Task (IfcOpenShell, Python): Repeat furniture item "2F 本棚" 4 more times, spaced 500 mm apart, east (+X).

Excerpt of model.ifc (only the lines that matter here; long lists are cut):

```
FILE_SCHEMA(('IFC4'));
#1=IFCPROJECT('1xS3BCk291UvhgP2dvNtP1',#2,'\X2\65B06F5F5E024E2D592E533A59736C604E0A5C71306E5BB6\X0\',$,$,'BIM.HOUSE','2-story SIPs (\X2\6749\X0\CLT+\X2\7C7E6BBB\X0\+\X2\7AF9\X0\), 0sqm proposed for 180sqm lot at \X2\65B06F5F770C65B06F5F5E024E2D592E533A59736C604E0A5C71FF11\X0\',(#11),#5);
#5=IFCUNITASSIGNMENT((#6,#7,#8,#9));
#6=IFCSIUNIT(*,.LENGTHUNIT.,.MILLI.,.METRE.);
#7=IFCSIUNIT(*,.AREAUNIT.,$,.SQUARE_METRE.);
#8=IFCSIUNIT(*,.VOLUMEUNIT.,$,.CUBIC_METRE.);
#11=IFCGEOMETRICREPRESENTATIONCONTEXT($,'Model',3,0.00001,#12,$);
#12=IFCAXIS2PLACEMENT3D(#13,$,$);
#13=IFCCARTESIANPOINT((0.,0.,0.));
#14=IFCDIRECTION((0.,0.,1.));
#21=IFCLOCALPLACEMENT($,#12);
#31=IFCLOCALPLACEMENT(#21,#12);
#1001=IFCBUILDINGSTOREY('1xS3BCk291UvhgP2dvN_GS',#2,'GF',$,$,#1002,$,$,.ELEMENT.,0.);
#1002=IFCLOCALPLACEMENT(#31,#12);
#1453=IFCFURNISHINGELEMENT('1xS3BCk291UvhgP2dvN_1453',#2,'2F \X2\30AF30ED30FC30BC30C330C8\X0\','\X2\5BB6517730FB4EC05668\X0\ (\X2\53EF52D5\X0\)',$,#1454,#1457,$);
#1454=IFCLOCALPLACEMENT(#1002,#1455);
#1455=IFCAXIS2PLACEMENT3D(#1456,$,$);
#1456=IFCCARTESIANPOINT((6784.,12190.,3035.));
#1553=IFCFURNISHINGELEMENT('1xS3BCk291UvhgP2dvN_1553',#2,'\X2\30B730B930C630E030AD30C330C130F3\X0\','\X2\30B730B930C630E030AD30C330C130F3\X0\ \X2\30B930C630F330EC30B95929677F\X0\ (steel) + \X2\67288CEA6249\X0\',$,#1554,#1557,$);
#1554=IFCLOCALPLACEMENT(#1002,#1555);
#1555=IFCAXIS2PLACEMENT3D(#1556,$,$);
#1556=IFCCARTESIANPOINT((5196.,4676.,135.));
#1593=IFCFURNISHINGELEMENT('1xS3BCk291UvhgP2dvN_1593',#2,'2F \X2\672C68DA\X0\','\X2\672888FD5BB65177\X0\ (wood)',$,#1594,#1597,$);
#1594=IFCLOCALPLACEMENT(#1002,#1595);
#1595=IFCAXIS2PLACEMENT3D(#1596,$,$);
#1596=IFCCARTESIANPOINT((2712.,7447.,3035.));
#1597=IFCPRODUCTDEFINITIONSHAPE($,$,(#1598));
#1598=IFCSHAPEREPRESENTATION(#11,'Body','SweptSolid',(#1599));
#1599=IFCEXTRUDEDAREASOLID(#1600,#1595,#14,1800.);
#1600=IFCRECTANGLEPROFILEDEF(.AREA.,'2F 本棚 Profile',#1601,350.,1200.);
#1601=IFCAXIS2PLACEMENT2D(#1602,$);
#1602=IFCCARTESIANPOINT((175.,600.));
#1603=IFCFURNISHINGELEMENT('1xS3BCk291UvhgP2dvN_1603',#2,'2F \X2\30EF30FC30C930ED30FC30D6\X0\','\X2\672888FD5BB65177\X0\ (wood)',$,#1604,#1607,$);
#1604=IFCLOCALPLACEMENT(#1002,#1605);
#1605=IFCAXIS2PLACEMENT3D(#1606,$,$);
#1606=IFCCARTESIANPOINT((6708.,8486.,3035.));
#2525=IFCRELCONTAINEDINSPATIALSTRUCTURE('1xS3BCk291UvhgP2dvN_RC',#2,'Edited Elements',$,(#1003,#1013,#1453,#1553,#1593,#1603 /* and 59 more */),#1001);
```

```python
import numpy as np
import ifcopenshell
import ifcopenshell.api.geometry
import ifcopenshell.api.root
import ifcopenshell.util.element
import ifcopenshell.util.placement

model = ifcopenshell.open("model.ifc")


def reuse_history(source, copy):
    """copy_class also copies each property set's owner history, people and application; keep the originals."""
    for rel in copy.IsDefinedBy:
        if rel.is_a("IfcRelDefinesByProperties") and (history := rel.RelatingPropertyDefinition.OwnerHistory):
            rel.RelatingPropertyDefinition.OwnerHistory = source.OwnerHistory
            ifcopenshell.util.element.remove_deep2(model, history)


source = model.by_id(1593)
base = ifcopenshell.util.placement.get_local_placement(source.ObjectPlacement)
step = np.array([1.0, 0.0, 0.0]) * 500.0

for i in range(1, 5):
    copy = ifcopenshell.api.root.copy_class(model, product=source)
    copy.Representation = ifcopenshell.util.element.copy_deep(
        model, source.Representation, exclude=["IfcGeometricRepresentationContext", "IfcRepresentationMap"]
    )
    reuse_history(source, copy)
    matrix = base.copy()
    matrix[:3, 3] += i * step
    print("added at", matrix[:3, 3].round(3) + 0.0)
    ifcopenshell.api.geometry.edit_object_placement(model, product=copy, matrix=matrix, is_si=False)

model.write("model_v2.ifc")
```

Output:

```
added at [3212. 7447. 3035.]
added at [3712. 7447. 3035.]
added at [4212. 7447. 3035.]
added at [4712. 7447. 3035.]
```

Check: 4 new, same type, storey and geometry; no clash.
